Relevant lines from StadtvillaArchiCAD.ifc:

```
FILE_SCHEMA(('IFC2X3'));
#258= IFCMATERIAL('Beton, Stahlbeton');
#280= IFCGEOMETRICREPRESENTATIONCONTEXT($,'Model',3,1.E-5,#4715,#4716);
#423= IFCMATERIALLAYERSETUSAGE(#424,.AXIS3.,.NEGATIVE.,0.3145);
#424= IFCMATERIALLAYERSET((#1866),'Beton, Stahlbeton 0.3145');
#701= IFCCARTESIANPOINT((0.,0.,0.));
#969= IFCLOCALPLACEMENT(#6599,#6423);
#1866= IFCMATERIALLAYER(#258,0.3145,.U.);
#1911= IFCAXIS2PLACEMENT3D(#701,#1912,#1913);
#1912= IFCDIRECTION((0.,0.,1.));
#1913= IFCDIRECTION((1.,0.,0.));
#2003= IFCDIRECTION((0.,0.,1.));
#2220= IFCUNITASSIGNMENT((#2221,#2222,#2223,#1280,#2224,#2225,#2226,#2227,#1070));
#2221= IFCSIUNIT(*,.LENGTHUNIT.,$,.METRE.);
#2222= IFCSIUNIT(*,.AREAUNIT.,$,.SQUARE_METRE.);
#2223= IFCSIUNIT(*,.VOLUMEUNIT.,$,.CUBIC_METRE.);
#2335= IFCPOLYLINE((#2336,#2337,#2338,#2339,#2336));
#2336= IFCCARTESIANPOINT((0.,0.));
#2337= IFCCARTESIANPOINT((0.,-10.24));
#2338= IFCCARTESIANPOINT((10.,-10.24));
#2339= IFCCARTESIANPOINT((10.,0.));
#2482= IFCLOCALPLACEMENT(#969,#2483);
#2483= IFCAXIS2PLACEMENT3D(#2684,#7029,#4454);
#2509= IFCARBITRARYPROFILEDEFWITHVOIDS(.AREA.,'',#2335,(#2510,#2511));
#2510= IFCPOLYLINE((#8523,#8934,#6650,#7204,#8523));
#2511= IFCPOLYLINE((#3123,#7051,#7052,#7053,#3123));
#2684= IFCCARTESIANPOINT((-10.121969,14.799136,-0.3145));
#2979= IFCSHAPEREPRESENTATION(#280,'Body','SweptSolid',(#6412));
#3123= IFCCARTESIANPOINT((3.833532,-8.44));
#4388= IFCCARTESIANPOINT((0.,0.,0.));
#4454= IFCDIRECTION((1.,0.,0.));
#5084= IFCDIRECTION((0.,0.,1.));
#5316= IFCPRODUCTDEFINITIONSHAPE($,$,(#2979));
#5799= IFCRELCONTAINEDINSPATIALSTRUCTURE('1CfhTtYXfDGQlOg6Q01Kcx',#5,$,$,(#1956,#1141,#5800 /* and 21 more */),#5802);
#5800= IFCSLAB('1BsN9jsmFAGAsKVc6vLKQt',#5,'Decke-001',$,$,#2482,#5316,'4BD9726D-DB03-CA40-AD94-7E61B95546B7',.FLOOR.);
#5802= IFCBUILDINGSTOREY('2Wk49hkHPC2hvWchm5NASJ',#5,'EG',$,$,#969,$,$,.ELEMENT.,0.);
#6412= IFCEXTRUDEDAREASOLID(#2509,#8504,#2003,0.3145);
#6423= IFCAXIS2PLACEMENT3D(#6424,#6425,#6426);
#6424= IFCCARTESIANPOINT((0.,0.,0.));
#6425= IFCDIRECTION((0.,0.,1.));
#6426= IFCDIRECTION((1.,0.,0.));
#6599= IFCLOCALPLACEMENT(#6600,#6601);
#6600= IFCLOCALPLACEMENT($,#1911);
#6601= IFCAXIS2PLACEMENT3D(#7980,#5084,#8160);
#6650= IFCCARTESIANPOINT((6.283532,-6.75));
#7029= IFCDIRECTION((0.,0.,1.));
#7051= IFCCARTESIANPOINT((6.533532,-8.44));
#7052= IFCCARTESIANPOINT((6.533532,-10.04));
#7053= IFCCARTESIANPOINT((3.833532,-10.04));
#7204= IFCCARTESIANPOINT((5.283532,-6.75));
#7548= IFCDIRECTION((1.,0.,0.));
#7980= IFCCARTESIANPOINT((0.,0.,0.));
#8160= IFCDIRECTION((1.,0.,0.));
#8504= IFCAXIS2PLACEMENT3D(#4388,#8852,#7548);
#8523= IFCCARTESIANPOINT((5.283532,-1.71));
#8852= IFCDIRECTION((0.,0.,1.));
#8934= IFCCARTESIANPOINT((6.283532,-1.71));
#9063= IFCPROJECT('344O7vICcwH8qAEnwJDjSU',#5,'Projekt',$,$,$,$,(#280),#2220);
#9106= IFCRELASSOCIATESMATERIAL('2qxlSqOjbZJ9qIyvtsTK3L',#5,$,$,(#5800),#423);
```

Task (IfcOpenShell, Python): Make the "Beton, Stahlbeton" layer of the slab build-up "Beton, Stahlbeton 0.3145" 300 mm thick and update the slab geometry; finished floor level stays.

```python
import ifcopenshell
import ifcopenshell.util.element
import ifcopenshell.util.unit

model = ifcopenshell.open("StadtvillaArchiCAD.ifc")
unit_scale = ifcopenshell.util.unit.calculate_unit_scale(model)

layer_set = model.by_id(424)
layer = next(l for l in layer_set.MaterialLayers if l.Material and l.Material.Name == "Beton, Stahlbeton")
change = 0.3 / unit_scale - layer.LayerThickness
layer.LayerThickness += change

# Geometry does not follow the layer set by itself.
slabs = [e for e in ifcopenshell.util.element.get_elements_by_material(model, layer_set) if e.is_a("IfcSlab")]
for slab in sorted(slabs, key=lambda e: e.id()):
    body = next(r for r in slab.Representation.Representations if r.RepresentationIdentifier == "Body")
    solid = body.Items[0]
    old_depth = solid.Depth
    solid.Depth += change
    # Extruded upwards: lower the start of the extrusion so the top stays.
    x, y, z = solid.Position.Location.Coordinates
    solid.Position.Location = model.createIfcCartesianPoint((x, y, z - change))
    print(slab.id(), f"{old_depth:g} -> {solid.Depth:g}")

model.write("StadtvillaArchiCAD_rev.ifc")
```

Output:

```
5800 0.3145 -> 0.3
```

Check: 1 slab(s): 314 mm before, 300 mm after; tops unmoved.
